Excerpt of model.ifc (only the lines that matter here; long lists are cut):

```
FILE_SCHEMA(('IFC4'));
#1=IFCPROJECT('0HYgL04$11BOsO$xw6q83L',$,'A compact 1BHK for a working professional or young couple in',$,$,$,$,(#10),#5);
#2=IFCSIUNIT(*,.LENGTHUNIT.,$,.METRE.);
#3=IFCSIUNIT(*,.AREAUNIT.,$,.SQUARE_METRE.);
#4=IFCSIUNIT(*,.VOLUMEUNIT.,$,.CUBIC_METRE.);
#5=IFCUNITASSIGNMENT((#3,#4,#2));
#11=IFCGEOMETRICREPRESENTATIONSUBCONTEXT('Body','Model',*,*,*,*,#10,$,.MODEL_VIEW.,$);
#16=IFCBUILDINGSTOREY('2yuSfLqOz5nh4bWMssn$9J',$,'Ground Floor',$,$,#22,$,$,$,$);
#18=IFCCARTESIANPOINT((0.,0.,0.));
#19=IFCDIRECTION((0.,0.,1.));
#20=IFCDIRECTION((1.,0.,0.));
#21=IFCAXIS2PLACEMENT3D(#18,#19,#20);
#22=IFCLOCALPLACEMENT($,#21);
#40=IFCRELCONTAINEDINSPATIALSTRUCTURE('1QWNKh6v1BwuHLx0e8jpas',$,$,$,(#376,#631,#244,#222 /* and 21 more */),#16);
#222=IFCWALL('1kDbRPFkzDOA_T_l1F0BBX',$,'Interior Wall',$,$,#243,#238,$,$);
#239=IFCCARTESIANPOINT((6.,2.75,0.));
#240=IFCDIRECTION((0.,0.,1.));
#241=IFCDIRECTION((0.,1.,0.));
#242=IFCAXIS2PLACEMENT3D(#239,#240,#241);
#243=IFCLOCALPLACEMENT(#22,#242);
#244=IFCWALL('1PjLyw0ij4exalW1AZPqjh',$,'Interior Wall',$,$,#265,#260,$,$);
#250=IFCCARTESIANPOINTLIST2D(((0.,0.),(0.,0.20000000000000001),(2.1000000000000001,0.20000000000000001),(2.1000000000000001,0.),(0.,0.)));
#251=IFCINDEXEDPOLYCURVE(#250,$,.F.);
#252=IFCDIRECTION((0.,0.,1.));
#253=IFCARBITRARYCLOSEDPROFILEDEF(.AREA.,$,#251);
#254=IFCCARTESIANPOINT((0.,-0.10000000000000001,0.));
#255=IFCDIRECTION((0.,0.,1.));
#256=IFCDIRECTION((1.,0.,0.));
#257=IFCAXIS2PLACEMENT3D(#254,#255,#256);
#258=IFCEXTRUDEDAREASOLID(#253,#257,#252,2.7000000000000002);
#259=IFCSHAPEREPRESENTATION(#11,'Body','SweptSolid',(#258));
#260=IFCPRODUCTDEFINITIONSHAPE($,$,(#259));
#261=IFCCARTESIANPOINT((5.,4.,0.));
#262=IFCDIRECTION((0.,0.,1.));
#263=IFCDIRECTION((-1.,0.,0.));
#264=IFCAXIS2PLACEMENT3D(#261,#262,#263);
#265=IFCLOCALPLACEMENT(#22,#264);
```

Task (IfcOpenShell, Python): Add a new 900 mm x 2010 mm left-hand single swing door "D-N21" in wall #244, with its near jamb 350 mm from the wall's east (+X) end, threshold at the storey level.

```python
import numpy as np
import ifcopenshell
import ifcopenshell.api.feature
import ifcopenshell.api.geometry
import ifcopenshell.api.root
import ifcopenshell.api.spatial
import ifcopenshell.geom
import ifcopenshell.util.element
import ifcopenshell.util.placement
import ifcopenshell.util.representation
import ifcopenshell.util.shape
import ifcopenshell.util.unit

model = ifcopenshell.open("model.ifc")
unit_scale = ifcopenshell.util.unit.calculate_unit_scale(model)
settings = ifcopenshell.geom.settings()


def volume(element):
    """Net volume in cubic metres, openings subtracted."""
    shape = ifcopenshell.geom.create_shape(settings, element)
    return ifcopenshell.util.shape.get_volume(shape.geometry)


wall = model.by_id(244)
storey = ifcopenshell.util.element.get_container(wall, ifc_class="IfcBuildingStorey")
context = ifcopenshell.util.representation.get_context(model, "Model", "Body", "MODEL_VIEW")
before = volume(wall)

width, height, from_end, sill = 0.9, 2.01, 0.35, 0.0  # metres

# The wall runs along its own X axis, and the end named is its -X end.
wall_shape = ifcopenshell.geom.create_shape(settings, wall)
x, y, z = ifcopenshell.util.shape.get_vertices(wall_shape.geometry).T
start = x.min() + from_end
face, thickness = float(y.min()), float(y.max() - y.min())
wall_matrix = ifcopenshell.util.placement.get_local_placement(wall.ObjectPlacement)
level = ifcopenshell.util.placement.get_local_placement(storey.ObjectPlacement)[2, 3]


def in_wall(x, y):
    """Placement at x, y metres in the wall's axes, at sill height."""
    matrix = wall_matrix.copy()
    matrix[:, 3] = wall_matrix @ np.array([x / unit_scale, y / unit_scale, 0.0, 1.0])
    matrix[2, 3] = level + sill / unit_scale
    return matrix


# Opening: a box that overshoots both wall faces by 50 mm.
opening = ifcopenshell.api.root.create_entity(model, ifc_class="IfcOpeningElement", predefined_type="OPENING")
box = ifcopenshell.api.geometry.add_wall_representation(
    model, context=context, length=width, height=height, thickness=thickness + 0.1
)
ifcopenshell.api.geometry.assign_representation(model, product=opening, representation=box)
ifcopenshell.api.geometry.edit_object_placement(model, product=opening, matrix=in_wall(start, face - 0.05), is_si=False)
ifcopenshell.api.feature.add_feature(model, feature=opening, element=wall)

door = ifcopenshell.api.root.create_entity(model, ifc_class="IfcDoor", name="D-N21", predefined_type="DOOR")
door.OverallWidth, door.OverallHeight = width / unit_scale, height / unit_scale
door.OperationType = "SINGLE_SWING_LEFT"
body = ifcopenshell.api.geometry.add_door_representation(
    model,
    context=context,
    overall_width=door.OverallWidth,
    overall_height=door.OverallHeight,
    operation_type="SINGLE_SWING_LEFT",
    lining_properties={"LiningDepth": thickness / unit_scale, "ThresholdDepth": thickness / unit_scale},
)
ifcopenshell.api.geometry.assign_representation(model, product=door, representation=body)
ifcopenshell.api.spatial.assign_container(model, products=[door], relating_structure=storey)
ifcopenshell.api.feature.add_filling(model, opening=opening, element=door)

# The lining spans the wall, so the door starts at the wall face.
ifcopenshell.api.geometry.edit_object_placement(model, product=door, matrix=in_wall(start, face), is_si=False)

after = volume(wall)

print(f"wall volume {before:.3f} -> {after:.3f} m3")

model.write("model-out.ifc")
```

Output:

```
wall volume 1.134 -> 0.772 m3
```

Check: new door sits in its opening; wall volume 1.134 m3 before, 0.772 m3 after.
